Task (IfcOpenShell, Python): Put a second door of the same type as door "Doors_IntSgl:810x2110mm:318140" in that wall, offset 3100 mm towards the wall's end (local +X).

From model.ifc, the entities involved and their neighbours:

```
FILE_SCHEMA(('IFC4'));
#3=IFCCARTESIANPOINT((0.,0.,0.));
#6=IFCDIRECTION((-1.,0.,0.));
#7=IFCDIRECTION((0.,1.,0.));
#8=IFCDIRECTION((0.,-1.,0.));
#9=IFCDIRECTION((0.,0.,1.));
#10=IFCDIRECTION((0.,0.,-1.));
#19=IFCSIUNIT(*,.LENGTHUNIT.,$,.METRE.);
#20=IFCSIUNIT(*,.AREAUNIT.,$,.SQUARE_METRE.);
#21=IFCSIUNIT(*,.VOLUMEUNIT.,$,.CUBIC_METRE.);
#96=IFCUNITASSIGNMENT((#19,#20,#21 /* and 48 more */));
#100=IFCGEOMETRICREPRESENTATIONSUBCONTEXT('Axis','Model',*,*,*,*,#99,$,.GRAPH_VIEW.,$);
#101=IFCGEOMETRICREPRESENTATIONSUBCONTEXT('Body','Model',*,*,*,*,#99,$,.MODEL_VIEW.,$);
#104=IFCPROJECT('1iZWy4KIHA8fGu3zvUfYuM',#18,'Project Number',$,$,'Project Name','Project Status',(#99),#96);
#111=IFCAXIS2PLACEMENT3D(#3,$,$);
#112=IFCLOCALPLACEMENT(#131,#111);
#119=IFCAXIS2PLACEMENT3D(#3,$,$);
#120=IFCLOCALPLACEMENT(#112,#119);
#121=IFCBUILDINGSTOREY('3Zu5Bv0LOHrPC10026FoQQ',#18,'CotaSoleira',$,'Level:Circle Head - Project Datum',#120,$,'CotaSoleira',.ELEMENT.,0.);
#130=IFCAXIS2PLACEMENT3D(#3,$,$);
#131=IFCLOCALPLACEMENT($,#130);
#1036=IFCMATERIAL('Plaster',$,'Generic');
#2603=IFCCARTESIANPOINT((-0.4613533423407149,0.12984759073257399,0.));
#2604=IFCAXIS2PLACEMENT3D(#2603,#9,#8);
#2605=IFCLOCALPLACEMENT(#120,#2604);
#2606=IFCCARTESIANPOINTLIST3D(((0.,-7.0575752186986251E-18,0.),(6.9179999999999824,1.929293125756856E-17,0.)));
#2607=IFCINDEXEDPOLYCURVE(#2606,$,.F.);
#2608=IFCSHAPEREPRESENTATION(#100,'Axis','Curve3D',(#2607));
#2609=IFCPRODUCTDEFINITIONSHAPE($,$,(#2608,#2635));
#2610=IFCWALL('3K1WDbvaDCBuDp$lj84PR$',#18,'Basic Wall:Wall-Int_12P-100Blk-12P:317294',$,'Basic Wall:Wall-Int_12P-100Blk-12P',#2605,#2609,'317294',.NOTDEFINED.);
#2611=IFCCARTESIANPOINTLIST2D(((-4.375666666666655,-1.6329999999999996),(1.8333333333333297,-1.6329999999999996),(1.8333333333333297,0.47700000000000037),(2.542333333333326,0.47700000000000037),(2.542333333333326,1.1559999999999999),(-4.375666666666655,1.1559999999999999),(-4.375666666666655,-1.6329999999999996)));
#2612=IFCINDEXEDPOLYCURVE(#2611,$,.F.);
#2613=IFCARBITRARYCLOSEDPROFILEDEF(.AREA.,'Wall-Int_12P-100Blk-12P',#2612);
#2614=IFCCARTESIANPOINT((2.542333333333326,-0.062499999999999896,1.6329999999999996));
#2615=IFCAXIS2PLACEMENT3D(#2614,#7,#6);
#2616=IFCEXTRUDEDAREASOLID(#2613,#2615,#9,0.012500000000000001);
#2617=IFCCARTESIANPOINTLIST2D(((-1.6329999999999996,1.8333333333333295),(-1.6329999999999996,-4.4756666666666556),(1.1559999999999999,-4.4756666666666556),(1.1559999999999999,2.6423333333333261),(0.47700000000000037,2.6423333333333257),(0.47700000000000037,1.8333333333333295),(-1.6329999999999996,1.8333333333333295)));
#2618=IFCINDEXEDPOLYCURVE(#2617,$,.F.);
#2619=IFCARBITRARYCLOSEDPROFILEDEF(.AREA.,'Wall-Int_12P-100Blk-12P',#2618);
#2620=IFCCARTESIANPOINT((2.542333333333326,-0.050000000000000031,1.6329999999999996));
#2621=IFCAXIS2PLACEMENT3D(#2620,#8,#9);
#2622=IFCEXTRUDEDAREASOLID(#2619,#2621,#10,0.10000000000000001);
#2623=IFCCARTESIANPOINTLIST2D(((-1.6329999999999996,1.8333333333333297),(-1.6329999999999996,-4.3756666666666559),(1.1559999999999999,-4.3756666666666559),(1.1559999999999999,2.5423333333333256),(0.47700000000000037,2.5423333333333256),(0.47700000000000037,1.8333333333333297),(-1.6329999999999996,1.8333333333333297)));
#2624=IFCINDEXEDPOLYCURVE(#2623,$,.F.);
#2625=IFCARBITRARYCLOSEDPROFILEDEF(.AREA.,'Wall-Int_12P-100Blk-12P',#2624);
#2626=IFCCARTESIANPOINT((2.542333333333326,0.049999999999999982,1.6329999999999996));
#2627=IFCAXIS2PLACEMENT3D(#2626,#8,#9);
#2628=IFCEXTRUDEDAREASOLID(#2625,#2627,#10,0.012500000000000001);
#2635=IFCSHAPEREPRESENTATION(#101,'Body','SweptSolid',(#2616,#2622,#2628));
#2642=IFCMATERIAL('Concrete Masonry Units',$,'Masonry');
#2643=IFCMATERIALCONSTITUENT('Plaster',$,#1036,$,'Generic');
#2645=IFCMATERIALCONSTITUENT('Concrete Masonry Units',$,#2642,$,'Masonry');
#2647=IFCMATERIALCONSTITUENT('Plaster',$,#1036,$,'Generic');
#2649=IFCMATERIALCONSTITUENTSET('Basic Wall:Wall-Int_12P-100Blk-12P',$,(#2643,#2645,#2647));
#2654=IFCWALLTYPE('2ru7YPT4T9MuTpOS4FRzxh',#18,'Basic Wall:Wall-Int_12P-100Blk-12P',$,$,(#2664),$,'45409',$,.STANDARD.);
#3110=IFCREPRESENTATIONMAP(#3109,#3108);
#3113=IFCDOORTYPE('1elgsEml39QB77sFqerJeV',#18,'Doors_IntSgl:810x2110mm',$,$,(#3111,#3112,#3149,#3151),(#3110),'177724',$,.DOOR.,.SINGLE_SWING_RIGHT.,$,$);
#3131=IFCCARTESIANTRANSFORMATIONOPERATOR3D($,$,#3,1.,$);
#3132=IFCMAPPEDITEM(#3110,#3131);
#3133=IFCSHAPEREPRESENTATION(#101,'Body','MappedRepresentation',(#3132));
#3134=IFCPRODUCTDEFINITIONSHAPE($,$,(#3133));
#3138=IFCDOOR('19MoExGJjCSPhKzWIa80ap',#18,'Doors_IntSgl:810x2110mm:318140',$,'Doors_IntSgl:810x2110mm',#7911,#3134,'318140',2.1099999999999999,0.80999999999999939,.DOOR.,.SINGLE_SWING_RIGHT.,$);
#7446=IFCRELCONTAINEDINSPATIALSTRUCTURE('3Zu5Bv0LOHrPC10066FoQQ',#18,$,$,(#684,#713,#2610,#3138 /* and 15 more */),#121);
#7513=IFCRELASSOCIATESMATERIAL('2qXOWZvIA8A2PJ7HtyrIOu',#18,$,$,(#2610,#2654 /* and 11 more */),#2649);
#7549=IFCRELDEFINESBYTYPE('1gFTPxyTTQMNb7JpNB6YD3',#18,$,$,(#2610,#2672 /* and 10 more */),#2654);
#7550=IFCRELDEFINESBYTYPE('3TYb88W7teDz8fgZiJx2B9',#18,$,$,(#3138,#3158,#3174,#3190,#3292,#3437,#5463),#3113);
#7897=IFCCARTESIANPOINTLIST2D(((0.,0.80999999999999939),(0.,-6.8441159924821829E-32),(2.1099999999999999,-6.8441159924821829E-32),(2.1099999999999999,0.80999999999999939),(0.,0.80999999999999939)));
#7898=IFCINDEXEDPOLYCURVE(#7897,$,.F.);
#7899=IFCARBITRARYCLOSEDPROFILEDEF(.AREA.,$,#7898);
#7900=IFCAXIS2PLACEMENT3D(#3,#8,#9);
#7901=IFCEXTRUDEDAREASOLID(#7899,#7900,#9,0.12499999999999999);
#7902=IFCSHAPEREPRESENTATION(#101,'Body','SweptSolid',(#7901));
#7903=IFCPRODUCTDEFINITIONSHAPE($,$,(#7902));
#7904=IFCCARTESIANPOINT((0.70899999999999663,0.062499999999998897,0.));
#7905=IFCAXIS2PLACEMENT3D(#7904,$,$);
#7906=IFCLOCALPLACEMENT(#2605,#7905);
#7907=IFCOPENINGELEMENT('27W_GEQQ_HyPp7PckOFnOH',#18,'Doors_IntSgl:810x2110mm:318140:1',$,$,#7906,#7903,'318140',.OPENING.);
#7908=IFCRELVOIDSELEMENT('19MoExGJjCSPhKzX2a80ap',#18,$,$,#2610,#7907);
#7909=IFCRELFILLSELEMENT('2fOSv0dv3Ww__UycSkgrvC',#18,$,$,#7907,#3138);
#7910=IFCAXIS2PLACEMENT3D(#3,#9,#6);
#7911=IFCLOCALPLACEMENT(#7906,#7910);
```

```python
import ifcopenshell
import ifcopenshell.api.feature
import ifcopenshell.api.geometry
import ifcopenshell.api.root
import ifcopenshell.geom
import ifcopenshell.util.element
import ifcopenshell.util.placement
import ifcopenshell.util.shape
import ifcopenshell.util.unit

model = ifcopenshell.open("model.ifc")
unit_scale = ifcopenshell.util.unit.calculate_unit_scale(model)
settings = ifcopenshell.geom.settings()


def volume(element):
    """Net volume in cubic metres, openings subtracted."""
    shape = ifcopenshell.geom.create_shape(settings, element)
    return ifcopenshell.util.shape.get_volume(shape.geometry)


def reuse_history(source, copy):
    """copy_class also copies each property set's owner history, people and application; keep the originals."""
    for rel in copy.IsDefinedBy:
        if rel.is_a("IfcRelDefinesByProperties") and (history := rel.RelatingPropertyDefinition.OwnerHistory):
            rel.RelatingPropertyDefinition.OwnerHistory = source.OwnerHistory
            ifcopenshell.util.element.remove_deep2(model, history)


door = model.by_guid("19MoExGJjCSPhKzWIa80ap")
opening = door.FillsVoids[0].RelatingOpeningElement
wall = opening.VoidsElements[0].RelatingBuildingElement
before = volume(wall)
shift = ifcopenshell.util.placement.get_local_placement(wall.ObjectPlacement)[:3, 0] * 3.1 / unit_scale

# copy_class copies the void relationship, type, container and properties, but no geometry.
new_opening = ifcopenshell.api.root.copy_class(model, product=opening)
new_opening.Representation = ifcopenshell.util.element.copy_deep(
    model, opening.Representation, exclude=["IfcGeometricRepresentationContext", "IfcRepresentationMap"]
)
new_opening.Name = "Doors_IntSgl:810x2110mm"
new_opening.Tag = None
new_door = ifcopenshell.api.root.copy_class(model, product=door)
new_door.Representation = ifcopenshell.util.element.copy_deep(
    model, door.Representation, exclude=["IfcGeometricRepresentationContext", "IfcRepresentationMap"]
)
new_door.Name = "Doors_IntSgl:810x2110mm"
new_door.Tag = None
reuse_history(door, new_door)
ifcopenshell.api.feature.add_filling(model, opening=new_opening, element=new_door)

for old, new in ((opening, new_opening), (door, new_door)):
    matrix = ifcopenshell.util.placement.get_local_placement(old.ObjectPlacement)
    matrix[:3, 3] += shift
    ifcopenshell.api.geometry.edit_object_placement(model, product=new, matrix=matrix, is_si=False)

after = volume(wall)

print(f"wall volume {before:.3f} -> {after:.3f} m3")

model.write("model_v2.ifc")
```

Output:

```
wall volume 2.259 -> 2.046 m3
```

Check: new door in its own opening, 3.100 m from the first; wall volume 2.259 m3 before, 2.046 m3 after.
